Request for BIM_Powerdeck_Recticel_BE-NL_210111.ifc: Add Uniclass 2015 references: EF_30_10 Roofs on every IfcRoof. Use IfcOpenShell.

First a look at what the model holds.

```python
import ifcopenshell

model = ifcopenshell.open("BIM_Powerdeck_Recticel_BE-NL_210111.ifc")
print(model.schema)
print("classifications:", [c.Name for c in model.by_type("IfcClassification")])
for ifc_class in ("IfcDoor", "IfcRoof", "IfcStair", "IfcWall", "IfcWindow"):
    print(ifc_class, len(model.by_type(ifc_class)))
```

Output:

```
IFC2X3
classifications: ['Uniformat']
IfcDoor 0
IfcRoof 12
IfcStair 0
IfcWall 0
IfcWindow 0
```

```python
import ifcopenshell
import ifcopenshell.api.classification

model = ifcopenshell.open("BIM_Powerdeck_Recticel_BE-NL_210111.ifc")

# IFC2X3 requires Source and Edition and has no link from the project to the system.
system = model.create_entity("IfcClassification", Source="NBS", Edition="2015", Name="Uniclass 2015")

codes = {
    "IfcRoof": ("EF_30_10", "Roofs"),
}
for ifc_class, (code, name) in codes.items():
    products = model.by_type(ifc_class)
    ifcopenshell.api.classification.add_reference(
        model, products=products, classification=system, identification=code, name=name
    )
    print(code, len(products))

model.write("BIM_Powerdeck_Recticel_BE-NL_210111_v2.ifc")
```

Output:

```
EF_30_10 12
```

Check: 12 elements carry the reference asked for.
